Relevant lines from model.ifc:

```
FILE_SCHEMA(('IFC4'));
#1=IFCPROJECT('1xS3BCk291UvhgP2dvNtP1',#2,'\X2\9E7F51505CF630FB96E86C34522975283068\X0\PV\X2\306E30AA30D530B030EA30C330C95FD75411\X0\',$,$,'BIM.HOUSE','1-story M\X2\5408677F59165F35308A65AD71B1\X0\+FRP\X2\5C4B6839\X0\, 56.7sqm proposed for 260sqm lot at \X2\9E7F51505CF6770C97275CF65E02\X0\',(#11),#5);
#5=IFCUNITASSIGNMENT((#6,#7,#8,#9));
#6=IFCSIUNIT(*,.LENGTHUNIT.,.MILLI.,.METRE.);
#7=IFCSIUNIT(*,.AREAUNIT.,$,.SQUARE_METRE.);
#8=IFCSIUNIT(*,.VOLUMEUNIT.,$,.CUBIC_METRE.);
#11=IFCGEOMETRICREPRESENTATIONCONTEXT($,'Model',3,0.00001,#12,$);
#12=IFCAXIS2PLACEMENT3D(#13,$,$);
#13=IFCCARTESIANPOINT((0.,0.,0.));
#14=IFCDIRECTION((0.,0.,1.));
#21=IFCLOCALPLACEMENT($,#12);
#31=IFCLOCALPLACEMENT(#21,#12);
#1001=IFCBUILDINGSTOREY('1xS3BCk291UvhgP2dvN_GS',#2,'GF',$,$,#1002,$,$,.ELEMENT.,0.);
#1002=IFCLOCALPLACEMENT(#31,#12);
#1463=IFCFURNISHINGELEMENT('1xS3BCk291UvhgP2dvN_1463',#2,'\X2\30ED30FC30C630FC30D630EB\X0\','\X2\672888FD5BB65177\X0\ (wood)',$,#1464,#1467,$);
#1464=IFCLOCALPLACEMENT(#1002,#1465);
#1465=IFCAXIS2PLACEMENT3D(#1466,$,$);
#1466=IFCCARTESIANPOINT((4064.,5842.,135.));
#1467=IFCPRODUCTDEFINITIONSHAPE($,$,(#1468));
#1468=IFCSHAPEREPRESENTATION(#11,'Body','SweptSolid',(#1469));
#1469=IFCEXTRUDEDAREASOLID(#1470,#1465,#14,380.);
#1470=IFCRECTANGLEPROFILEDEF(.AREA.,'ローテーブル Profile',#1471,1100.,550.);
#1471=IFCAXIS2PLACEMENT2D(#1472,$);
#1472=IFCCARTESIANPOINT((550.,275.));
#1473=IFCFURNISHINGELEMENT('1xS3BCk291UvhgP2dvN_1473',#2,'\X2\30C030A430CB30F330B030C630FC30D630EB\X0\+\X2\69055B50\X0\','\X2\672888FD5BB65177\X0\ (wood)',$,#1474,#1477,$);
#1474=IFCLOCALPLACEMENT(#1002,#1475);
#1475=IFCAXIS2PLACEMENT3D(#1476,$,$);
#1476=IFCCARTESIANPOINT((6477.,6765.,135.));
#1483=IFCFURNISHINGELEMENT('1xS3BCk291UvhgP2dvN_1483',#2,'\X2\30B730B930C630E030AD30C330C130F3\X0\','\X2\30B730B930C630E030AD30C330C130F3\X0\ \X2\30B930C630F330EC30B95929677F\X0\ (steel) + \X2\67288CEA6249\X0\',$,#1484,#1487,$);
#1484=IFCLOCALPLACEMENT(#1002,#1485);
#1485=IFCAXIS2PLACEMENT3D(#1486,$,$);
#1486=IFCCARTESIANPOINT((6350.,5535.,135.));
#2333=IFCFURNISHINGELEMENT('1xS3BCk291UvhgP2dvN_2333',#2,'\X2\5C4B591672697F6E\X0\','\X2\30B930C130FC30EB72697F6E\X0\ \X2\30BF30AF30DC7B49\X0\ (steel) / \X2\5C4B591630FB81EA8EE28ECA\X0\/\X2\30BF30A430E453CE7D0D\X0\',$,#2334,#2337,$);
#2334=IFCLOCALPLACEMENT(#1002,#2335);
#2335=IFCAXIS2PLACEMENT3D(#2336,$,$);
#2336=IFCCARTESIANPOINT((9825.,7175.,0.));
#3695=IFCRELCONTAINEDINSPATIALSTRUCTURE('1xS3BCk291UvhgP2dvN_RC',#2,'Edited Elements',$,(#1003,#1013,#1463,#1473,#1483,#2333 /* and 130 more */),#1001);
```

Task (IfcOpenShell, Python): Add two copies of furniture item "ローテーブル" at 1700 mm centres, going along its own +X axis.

```python
import ifcopenshell
import ifcopenshell.api.geometry
import ifcopenshell.api.root
import ifcopenshell.util.element
import ifcopenshell.util.placement
import ifcopenshell.util.unit

model = ifcopenshell.open("model.ifc")
unit_scale = ifcopenshell.util.unit.calculate_unit_scale(model)


def reuse_history(source, copy):
    """copy_class also copies each property set's owner history, people and application; keep the originals."""
    for rel in copy.IsDefinedBy:
        if rel.is_a("IfcRelDefinesByProperties") and (history := rel.RelatingPropertyDefinition.OwnerHistory):
            rel.RelatingPropertyDefinition.OwnerHistory = source.OwnerHistory
            ifcopenshell.util.element.remove_deep2(model, history)


source = model.by_id(1463)
base = ifcopenshell.util.placement.get_local_placement(source.ObjectPlacement)
step = base[:3, 0] * 1.7 / unit_scale

for i in range(1, 3):
    copy = ifcopenshell.api.root.copy_class(model, product=source)
    copy.Representation = ifcopenshell.util.element.copy_deep(
        model, source.Representation, exclude=["IfcGeometricRepresentationContext", "IfcRepresentationMap"]
    )
    reuse_history(source, copy)
    matrix = base.copy()
    matrix[:3, 3] += i * step
    print("added at", matrix[:3, 3].round(3) + 0.0)
    ifcopenshell.api.geometry.edit_object_placement(model, product=copy, matrix=matrix, is_si=False)

model.write("model-out.ifc")
```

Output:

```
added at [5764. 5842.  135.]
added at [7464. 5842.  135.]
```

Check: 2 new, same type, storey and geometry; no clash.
